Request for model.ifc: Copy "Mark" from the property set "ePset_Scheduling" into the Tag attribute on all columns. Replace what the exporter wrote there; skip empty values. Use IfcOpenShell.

First a look at what the model holds.

```python
import ifcopenshell
import ifcopenshell.util.element

model = ifcopenshell.open("model.ifc")
print(model.schema)
columns = model.by_type("IfcColumn")
print(len(columns), "columns")
for e in columns[:8]:
    source = ifcopenshell.util.element.get_pset(e, "ePset_Scheduling", "Mark")
    target = e.Tag
    print(e.id(), repr(source), repr(target), sep=" | ")
```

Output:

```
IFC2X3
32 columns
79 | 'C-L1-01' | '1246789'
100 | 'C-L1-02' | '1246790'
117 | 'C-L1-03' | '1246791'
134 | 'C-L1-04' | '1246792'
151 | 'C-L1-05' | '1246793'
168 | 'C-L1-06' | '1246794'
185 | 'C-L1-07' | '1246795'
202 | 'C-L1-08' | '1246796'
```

```python
import ifcopenshell
import ifcopenshell.util.element

model = ifcopenshell.open("model.ifc")

count = 0
for e in model.by_type("IfcColumn"):
    value = ifcopenshell.util.element.get_pset(e, "ePset_Scheduling", "Mark")
    current = e.Tag
    if not value or not value.strip() or current == value:
        continue
    e.Tag = value
    count += 1

print(count, "columns updated")

model.write("model_edited.ifc")
```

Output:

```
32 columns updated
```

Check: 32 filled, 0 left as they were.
